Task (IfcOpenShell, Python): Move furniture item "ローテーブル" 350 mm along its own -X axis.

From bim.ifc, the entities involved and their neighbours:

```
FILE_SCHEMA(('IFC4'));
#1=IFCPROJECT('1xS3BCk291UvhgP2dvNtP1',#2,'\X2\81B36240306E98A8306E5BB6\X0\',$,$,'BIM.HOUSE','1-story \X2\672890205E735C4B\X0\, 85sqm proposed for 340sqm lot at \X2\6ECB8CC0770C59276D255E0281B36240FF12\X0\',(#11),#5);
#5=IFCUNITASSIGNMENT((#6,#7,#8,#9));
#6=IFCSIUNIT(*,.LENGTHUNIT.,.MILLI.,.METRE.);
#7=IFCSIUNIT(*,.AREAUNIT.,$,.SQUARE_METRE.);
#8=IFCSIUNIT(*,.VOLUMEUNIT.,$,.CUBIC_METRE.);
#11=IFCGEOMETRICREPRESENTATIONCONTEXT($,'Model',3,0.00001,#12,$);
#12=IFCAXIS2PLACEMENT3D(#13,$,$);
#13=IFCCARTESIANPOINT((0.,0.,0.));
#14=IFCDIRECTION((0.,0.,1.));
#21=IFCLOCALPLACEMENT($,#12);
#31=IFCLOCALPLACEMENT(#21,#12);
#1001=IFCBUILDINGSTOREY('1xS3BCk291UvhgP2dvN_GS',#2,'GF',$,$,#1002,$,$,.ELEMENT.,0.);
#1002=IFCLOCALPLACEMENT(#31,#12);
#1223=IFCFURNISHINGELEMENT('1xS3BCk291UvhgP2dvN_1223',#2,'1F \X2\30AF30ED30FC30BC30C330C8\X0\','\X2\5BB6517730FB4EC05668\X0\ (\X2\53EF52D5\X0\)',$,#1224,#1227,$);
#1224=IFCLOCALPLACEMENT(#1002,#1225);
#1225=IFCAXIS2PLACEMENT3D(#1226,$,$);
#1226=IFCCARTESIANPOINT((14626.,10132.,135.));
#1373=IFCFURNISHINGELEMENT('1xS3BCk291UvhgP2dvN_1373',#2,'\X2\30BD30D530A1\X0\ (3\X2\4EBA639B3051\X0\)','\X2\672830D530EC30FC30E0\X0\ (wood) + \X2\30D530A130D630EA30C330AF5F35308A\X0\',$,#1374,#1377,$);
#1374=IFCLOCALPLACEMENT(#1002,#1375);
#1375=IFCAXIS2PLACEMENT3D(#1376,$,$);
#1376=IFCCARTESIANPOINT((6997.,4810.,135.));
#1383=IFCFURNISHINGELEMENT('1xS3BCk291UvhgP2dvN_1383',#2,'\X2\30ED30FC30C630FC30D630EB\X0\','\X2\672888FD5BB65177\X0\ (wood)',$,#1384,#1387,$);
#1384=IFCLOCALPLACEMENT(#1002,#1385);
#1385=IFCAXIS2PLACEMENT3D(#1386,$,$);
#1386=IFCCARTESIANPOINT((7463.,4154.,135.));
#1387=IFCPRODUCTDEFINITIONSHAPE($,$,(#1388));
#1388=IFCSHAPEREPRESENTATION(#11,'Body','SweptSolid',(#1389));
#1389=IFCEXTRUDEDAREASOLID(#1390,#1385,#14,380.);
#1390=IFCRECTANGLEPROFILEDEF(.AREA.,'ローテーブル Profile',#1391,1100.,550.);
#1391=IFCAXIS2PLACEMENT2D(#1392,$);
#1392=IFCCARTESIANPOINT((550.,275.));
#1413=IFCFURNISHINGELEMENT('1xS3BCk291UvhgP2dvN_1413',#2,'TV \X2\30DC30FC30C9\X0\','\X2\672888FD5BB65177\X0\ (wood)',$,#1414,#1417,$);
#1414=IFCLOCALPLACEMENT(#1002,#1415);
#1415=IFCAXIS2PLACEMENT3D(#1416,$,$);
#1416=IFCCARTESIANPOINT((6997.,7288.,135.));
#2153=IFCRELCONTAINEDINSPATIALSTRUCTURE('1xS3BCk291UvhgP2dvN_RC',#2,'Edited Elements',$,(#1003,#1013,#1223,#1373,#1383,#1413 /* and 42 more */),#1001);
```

```python
import ifcopenshell
import ifcopenshell.api.geometry
import ifcopenshell.util.placement

model = ifcopenshell.open("bim.ifc")

item = model.by_id(1383)
matrix = ifcopenshell.util.placement.get_local_placement(item.ObjectPlacement)
matrix[:3, 3] -= matrix[:3, 0] * 350.0
ifcopenshell.api.geometry.edit_object_placement(model, product=item, matrix=matrix, is_si=False)

print(ifcopenshell.util.placement.get_local_placement(item.ObjectPlacement).round(3) + 0.0)

model.write("bim_rev.ifc")
```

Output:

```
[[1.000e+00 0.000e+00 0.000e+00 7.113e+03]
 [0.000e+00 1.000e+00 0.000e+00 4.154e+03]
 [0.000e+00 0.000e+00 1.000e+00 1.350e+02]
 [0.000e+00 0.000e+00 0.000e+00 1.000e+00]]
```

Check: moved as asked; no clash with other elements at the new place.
